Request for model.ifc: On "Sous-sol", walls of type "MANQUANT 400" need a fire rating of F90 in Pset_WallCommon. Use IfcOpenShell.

First a look at what the model holds.

```python
import ifcopenshell
import ifcopenshell.util.element

model = ifcopenshell.open("model.ifc")
print(model.schema)
storey = next(s for s in model.by_type("IfcBuildingStorey") if s.Name == "Sous-sol")
walls = [e for e in ifcopenshell.util.element.get_decomposition(storey) if e.is_a("IfcWall")]
seen = {}
for e in walls:
    element_type = ifcopenshell.util.element.get_type(e)
    key = (element_type.Name if element_type != e and element_type else None, ifcopenshell.util.element.get_pset(e, "Pset_WallCommon", "FireRating"))
    seen[key] = seen.get(key, 0) + 1
for (name, value), count in sorted(seen.items(), key=str):
    print(count, "x", name, "|", value)
```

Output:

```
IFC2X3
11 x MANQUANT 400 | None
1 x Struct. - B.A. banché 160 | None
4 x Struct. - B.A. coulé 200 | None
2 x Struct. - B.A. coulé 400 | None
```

```python
import ifcopenshell
import ifcopenshell.api.pset
import ifcopenshell.util.element

model = ifcopenshell.open("model.ifc")

storey = next(s for s in model.by_type("IfcBuildingStorey") if s.Name == "Sous-sol")
walls = [e for e in ifcopenshell.util.element.get_decomposition(storey) if e.is_a("IfcWall")]

count = 0
for e in walls:
    element_type = ifcopenshell.util.element.get_type(e)
    if element_type in (None, e) or element_type.Name != "MANQUANT 400":
        continue
    # add_pset returns the element's existing set when there is one.
    pset = ifcopenshell.api.pset.add_pset(model, product=e, name="Pset_WallCommon")
    ifcopenshell.api.pset.edit_pset(model, pset=pset, properties={"FireRating": "F90"})
    count += 1

print(count, "walls updated")

model.write("model_v2.ifc")
```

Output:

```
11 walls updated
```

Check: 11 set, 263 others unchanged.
